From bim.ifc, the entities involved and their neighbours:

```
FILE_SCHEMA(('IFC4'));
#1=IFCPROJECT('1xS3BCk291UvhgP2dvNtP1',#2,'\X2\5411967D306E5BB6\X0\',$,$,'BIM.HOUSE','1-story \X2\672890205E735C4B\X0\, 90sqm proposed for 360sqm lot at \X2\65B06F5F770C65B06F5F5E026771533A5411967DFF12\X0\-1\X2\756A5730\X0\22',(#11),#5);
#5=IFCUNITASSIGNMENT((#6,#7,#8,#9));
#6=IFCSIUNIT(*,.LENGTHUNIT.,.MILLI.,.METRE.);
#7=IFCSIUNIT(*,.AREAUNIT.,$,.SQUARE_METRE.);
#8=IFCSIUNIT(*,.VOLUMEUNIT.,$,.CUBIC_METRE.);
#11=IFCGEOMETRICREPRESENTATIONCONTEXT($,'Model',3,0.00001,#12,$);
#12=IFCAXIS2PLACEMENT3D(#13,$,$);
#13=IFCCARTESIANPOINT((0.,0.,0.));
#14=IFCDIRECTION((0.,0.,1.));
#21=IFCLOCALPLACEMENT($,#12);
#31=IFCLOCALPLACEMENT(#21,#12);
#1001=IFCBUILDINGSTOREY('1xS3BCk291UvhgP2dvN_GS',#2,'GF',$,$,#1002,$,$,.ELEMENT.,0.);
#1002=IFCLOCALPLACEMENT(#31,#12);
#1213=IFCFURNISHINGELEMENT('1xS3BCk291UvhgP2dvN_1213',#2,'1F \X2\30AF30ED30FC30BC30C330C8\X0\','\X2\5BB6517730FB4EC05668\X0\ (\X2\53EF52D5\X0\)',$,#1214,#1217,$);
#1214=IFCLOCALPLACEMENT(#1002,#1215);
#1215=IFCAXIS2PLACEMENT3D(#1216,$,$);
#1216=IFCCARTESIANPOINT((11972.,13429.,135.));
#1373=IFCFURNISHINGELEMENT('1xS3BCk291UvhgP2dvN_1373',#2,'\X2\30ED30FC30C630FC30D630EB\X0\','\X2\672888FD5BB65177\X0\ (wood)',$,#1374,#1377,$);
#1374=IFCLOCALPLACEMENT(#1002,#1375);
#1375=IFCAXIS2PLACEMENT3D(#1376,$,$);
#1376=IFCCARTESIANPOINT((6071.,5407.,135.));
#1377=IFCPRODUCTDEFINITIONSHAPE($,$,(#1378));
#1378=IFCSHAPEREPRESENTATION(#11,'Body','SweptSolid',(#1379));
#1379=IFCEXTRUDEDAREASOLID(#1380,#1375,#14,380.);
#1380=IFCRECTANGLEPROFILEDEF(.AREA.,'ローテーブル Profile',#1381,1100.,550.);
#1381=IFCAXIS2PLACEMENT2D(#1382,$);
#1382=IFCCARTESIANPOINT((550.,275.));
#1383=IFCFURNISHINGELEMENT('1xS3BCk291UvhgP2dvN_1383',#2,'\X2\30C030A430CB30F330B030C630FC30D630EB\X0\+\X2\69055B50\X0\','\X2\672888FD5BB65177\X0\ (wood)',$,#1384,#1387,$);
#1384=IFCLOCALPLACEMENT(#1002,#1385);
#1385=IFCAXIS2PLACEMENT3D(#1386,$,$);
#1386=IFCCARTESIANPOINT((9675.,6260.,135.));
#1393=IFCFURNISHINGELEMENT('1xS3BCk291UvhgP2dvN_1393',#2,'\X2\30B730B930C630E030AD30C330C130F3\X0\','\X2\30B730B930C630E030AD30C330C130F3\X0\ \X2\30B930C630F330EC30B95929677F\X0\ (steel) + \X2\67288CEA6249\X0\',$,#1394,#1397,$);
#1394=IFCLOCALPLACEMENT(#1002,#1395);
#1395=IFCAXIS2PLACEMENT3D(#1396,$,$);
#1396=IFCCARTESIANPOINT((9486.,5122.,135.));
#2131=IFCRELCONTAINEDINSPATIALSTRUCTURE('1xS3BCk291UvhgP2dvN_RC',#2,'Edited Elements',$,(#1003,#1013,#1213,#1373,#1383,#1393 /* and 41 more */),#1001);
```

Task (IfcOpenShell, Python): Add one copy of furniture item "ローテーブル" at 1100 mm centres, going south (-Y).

```python
import numpy as np
import ifcopenshell
import ifcopenshell.api.geometry
import ifcopenshell.api.root
import ifcopenshell.util.element
import ifcopenshell.util.placement
import ifcopenshell.util.unit

model = ifcopenshell.open("bim.ifc")
unit_scale = ifcopenshell.util.unit.calculate_unit_scale(model)


def reuse_history(source, copy):
    """copy_class also copies each property set's owner history, people and application; keep the originals."""
    for rel in copy.IsDefinedBy:
        if rel.is_a("IfcRelDefinesByProperties") and (history := rel.RelatingPropertyDefinition.OwnerHistory):
            rel.RelatingPropertyDefinition.OwnerHistory = source.OwnerHistory
            ifcopenshell.util.element.remove_deep2(model, history)


source = model.by_guid("1xS3BCk291UvhgP2dvN_1373")
base = ifcopenshell.util.placement.get_local_placement(source.ObjectPlacement)
step = np.array([0.0, -1.0, 0.0]) * 1.1 / unit_scale

for i in range(1, 2):
    copy = ifcopenshell.api.root.copy_class(model, product=source)
    copy.Representation = ifcopenshell.util.element.copy_deep(
        model, source.Representation, exclude=["IfcGeometricRepresentationContext", "IfcRepresentationMap"]
    )
    reuse_history(source, copy)
    matrix = base.copy()
    matrix[:3, 3] += i * step
    print("added at", matrix[:3, 3].round(3) + 0.0)
    ifcopenshell.api.geometry.edit_object_placement(model, product=copy, matrix=matrix, is_si=False)

model.write("bim_v2.ifc")
```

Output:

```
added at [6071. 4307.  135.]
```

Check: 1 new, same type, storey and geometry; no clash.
